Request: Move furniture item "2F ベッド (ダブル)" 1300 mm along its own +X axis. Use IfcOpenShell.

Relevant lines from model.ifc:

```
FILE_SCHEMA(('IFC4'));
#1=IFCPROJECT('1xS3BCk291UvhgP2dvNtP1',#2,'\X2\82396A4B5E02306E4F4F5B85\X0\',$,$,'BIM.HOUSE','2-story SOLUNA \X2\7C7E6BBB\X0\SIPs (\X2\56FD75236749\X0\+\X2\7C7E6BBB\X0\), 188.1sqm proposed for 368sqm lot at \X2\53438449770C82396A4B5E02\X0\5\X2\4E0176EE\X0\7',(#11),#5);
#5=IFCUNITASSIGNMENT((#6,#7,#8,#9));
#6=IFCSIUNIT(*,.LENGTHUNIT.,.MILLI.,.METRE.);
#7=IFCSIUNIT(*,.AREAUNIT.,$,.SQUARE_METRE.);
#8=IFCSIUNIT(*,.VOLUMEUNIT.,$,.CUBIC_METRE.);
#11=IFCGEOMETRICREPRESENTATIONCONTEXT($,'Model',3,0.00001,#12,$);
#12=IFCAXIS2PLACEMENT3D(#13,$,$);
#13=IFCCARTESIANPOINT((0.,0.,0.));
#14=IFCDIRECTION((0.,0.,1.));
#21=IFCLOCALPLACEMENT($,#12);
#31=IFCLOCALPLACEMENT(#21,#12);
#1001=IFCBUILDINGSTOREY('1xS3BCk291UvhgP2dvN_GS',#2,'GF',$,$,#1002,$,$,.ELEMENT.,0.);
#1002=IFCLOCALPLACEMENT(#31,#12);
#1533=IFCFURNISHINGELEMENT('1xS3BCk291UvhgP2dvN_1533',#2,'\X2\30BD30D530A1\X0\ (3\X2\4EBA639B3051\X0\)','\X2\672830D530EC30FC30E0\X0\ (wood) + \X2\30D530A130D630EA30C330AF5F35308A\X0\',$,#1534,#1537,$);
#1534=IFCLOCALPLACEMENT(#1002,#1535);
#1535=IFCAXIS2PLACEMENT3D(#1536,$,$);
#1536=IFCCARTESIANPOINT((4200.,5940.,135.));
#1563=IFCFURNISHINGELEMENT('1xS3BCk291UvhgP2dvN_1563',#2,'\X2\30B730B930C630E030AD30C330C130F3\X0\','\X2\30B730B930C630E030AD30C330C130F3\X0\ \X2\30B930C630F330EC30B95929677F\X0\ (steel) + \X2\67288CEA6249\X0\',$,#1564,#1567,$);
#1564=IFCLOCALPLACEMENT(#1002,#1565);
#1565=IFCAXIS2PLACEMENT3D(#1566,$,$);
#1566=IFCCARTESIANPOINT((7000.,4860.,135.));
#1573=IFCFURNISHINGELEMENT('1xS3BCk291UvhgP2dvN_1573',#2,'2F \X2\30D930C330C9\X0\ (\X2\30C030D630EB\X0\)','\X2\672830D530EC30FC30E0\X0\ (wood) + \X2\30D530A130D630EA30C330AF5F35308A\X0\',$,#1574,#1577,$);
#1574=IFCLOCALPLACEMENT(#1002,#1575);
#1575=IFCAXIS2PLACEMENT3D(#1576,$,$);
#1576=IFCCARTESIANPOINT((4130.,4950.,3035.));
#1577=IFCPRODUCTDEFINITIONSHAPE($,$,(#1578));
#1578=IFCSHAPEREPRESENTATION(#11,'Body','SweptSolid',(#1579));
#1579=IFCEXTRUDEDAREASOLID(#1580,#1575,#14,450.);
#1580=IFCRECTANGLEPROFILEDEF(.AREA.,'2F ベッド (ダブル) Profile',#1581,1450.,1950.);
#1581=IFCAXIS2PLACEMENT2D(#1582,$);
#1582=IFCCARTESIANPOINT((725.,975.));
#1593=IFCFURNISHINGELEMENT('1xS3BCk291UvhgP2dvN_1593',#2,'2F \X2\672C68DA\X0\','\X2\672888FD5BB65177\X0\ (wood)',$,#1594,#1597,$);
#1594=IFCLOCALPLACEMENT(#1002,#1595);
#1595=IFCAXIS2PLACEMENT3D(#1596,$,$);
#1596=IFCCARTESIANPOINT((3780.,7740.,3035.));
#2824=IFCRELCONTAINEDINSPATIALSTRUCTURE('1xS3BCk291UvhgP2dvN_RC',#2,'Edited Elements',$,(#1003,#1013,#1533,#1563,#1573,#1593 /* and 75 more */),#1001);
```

```python
import ifcopenshell
import ifcopenshell.api.geometry
import ifcopenshell.util.placement

model = ifcopenshell.open("model.ifc")

item = model.by_guid("1xS3BCk291UvhgP2dvN_1573")
matrix = ifcopenshell.util.placement.get_local_placement(item.ObjectPlacement)
matrix[:3, 3] += matrix[:3, 0] * 1300.0
ifcopenshell.api.geometry.edit_object_placement(model, product=item, matrix=matrix, is_si=False)

print(ifcopenshell.util.placement.get_local_placement(item.ObjectPlacement).round(3) + 0.0)

model.write("model_edited.ifc")
```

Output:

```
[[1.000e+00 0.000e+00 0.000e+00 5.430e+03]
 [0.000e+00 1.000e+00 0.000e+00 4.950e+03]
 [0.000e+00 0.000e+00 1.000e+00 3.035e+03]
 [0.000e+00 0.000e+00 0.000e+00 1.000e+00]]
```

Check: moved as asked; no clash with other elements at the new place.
